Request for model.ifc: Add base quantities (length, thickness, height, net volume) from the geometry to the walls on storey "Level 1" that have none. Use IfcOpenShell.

First a look at what the model holds.

```python
import ifcopenshell
import ifcopenshell.util.element
import ifcopenshell.util.unit

model = ifcopenshell.open("model.ifc")
print(model.schema)
for unit_type in ("LENGTHUNIT", "AREAUNIT", "VOLUMEUNIT"):
    print(unit_type, ifcopenshell.util.unit.calculate_unit_scale(model, unit_type))
storey = next(s for s in model.by_type("IfcBuildingStorey") if s.Name == "Level 1")
walls = [e for e in ifcopenshell.util.element.get_decomposition(storey) if e.is_a("IfcWall")]
for e in sorted(walls, key=lambda e: e.id()):
    print(e.id(), e.is_a(), e.Name, list(ifcopenshell.util.element.get_psets(e, qtos_only=True)), sep=" | ")
```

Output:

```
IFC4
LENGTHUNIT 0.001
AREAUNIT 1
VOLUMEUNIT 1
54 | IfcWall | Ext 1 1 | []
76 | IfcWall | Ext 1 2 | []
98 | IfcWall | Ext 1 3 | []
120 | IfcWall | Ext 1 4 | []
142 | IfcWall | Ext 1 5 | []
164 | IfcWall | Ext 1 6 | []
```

```python
import ifcopenshell
import ifcopenshell.api.pset
import ifcopenshell.geom
import ifcopenshell.util.element
import ifcopenshell.util.shape
import ifcopenshell.util.unit

model = ifcopenshell.open("model.ifc")
unit_scale = ifcopenshell.util.unit.calculate_unit_scale(model)
volume_scale = ifcopenshell.util.unit.calculate_unit_scale(model, "VOLUMEUNIT")
settings = ifcopenshell.geom.settings()

storey = next(s for s in model.by_type("IfcBuildingStorey") if s.Name == "Level 1")
walls = [e for e in ifcopenshell.util.element.get_decomposition(storey) if e.is_a("IfcWall")]

for e in sorted(walls, key=lambda e: e.id()):
    if ifcopenshell.util.element.get_psets(e, qtos_only=True, should_inherit=False):
        continue
    # Geometry comes back in metres, in the element's own axes.
    shape = ifcopenshell.geom.create_shape(settings, e)
    values = {
        "Length": ifcopenshell.util.shape.get_x(shape.geometry) / unit_scale,
        "Width": ifcopenshell.util.shape.get_y(shape.geometry) / unit_scale,
        "Height": ifcopenshell.util.shape.get_z(shape.geometry) / unit_scale,
        "NetVolume": ifcopenshell.util.shape.get_volume(shape.geometry) / volume_scale,
    }
    qto = ifcopenshell.api.pset.add_qto(model, product=e, name="Qto_WallBaseQuantities")
    ifcopenshell.api.pset.edit_qto(model, qto=qto, properties=values)
    print(e.id(), {k: round(v, 3) for k, v in values.items()})

model.write("model_rev.ifc")
```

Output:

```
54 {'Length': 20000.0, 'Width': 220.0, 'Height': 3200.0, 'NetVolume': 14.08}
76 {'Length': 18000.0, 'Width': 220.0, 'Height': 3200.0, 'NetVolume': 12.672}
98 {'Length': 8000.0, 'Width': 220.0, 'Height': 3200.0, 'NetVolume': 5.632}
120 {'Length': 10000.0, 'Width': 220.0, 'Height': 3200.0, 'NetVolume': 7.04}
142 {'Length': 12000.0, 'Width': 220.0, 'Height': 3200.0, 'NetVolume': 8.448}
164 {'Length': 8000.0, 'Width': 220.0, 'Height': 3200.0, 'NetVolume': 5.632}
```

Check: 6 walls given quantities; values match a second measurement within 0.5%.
